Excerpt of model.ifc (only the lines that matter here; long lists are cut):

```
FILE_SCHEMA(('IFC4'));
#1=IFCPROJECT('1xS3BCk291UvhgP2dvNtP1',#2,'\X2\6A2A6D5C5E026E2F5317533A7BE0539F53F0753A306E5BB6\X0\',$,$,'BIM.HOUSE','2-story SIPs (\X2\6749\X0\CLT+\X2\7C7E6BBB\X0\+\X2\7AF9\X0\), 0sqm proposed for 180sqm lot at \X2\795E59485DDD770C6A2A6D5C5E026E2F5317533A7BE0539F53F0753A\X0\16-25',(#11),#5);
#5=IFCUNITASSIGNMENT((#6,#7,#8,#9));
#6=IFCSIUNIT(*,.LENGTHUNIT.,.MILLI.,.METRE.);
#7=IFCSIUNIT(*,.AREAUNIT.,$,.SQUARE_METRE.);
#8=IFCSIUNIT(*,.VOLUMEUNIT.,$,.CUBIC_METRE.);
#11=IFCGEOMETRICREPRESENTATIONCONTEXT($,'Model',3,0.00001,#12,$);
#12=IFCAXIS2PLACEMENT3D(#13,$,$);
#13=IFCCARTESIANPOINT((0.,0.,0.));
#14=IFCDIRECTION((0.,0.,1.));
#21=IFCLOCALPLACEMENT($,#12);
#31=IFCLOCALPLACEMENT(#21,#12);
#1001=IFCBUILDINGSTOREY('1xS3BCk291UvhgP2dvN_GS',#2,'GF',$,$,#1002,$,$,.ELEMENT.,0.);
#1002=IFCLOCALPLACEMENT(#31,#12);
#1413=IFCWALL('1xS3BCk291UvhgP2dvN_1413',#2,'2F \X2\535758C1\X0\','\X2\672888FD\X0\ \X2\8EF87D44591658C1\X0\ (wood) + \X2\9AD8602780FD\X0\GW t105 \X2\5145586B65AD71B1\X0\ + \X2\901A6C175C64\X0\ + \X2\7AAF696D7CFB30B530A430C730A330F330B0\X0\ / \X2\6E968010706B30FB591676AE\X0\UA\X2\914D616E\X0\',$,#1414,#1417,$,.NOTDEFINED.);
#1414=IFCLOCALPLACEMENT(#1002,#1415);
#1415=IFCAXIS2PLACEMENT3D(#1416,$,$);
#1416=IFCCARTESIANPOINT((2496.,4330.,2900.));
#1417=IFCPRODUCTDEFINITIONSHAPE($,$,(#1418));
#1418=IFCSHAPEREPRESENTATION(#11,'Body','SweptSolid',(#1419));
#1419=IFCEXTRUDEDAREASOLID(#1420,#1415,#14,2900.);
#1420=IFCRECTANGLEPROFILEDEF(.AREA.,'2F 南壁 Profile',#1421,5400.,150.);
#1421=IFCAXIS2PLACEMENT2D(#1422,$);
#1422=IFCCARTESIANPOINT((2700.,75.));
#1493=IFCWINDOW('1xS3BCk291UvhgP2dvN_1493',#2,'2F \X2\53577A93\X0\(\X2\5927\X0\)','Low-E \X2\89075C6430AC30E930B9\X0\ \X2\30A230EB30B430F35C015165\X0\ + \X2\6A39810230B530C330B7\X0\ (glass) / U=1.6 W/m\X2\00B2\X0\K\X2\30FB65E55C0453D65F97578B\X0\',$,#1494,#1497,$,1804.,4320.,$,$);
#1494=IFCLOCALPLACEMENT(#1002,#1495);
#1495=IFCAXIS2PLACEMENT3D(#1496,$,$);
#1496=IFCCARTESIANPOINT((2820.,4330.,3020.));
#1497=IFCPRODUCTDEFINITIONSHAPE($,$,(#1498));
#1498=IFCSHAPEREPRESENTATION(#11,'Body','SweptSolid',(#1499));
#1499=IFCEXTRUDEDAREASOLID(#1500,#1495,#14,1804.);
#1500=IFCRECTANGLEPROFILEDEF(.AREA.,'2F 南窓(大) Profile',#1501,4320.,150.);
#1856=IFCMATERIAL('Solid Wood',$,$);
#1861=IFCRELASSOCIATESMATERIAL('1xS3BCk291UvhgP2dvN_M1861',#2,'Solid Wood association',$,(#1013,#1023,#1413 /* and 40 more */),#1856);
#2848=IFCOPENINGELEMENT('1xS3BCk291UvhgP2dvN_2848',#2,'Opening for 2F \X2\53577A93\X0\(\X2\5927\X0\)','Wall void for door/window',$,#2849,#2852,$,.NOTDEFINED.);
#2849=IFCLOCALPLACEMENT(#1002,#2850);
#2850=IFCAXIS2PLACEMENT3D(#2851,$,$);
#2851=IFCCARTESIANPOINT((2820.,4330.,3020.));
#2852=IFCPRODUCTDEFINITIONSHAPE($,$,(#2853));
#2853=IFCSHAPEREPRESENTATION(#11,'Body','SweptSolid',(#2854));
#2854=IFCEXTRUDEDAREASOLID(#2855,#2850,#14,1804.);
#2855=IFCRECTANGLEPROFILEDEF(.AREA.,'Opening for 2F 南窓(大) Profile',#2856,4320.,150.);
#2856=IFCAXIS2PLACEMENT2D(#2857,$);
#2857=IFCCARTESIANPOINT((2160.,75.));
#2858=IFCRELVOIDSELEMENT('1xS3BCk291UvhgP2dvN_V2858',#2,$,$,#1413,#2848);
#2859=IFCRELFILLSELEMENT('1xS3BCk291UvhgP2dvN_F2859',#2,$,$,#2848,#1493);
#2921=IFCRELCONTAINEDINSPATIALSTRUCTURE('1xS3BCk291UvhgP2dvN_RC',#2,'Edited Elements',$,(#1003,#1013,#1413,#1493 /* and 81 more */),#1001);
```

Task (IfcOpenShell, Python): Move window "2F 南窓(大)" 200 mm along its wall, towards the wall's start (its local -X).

```python
import ifcopenshell
import ifcopenshell.api.geometry
import ifcopenshell.util.placement
import ifcopenshell.util.unit

model = ifcopenshell.open("model.ifc")
unit_scale = ifcopenshell.util.unit.calculate_unit_scale(model)

window = model.by_guid("1xS3BCk291UvhgP2dvN_1493")
opening = window.FillsVoids[0].RelatingOpeningElement
wall = opening.VoidsElements[0].RelatingBuildingElement

wall_matrix = ifcopenshell.util.placement.get_local_placement(wall.ObjectPlacement)
shift = wall_matrix[:3, 0] * -0.2 / unit_scale
before = ifcopenshell.util.placement.get_local_placement(window.ObjectPlacement)[:3, 3].copy()

# The window is not placed relative to its opening, so move both.
for product in (opening, window):
    matrix = ifcopenshell.util.placement.get_local_placement(product.ObjectPlacement)
    matrix[:3, 3] += shift
    ifcopenshell.api.geometry.edit_object_placement(model, product=product, matrix=matrix, is_si=False)

after = ifcopenshell.util.placement.get_local_placement(window.ObjectPlacement)[:3, 3]
print("window moved by", (after - before).round(3) + 0.0)

model.write("model_v2.ifc")
```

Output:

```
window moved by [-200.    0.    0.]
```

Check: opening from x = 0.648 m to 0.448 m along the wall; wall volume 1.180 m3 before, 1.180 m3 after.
